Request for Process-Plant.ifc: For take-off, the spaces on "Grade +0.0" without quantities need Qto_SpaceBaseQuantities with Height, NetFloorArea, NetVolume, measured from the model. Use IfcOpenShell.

First a look at what the model holds.

```python
import ifcopenshell
import ifcopenshell.util.element
import ifcopenshell.util.unit

model = ifcopenshell.open("Process-Plant.ifc")
print(model.schema)
for unit_type in ("LENGTHUNIT", "AREAUNIT", "VOLUMEUNIT"):
    print(unit_type, ifcopenshell.util.unit.calculate_unit_scale(model, unit_type))
storey = next(s for s in model.by_type("IfcBuildingStorey") if s.Name == "Grade +0.0")
spaces = [e for e in ifcopenshell.util.element.get_decomposition(storey) if e.is_a("IfcSpace")]
for e in sorted(spaces, key=lambda e: e.id()):
    print(e.id(), e.is_a(), e.Name, list(ifcopenshell.util.element.get_psets(e, qtos_only=True)), sep=" | ")
```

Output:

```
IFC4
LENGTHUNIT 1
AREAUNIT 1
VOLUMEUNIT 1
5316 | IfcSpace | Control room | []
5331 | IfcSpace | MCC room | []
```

```python
import ifcopenshell
import ifcopenshell.api.pset
import ifcopenshell.geom
import ifcopenshell.util.element
import ifcopenshell.util.shape
import ifcopenshell.util.unit

model = ifcopenshell.open("Process-Plant.ifc")
unit_scale = ifcopenshell.util.unit.calculate_unit_scale(model)
area_scale = ifcopenshell.util.unit.calculate_unit_scale(model, "AREAUNIT")
volume_scale = ifcopenshell.util.unit.calculate_unit_scale(model, "VOLUMEUNIT")
settings = ifcopenshell.geom.settings()

storey = next(s for s in model.by_type("IfcBuildingStorey") if s.Name == "Grade +0.0")
spaces = [e for e in ifcopenshell.util.element.get_decomposition(storey) if e.is_a("IfcSpace")]

for e in sorted(spaces, key=lambda e: e.id()):
    if ifcopenshell.util.element.get_psets(e, qtos_only=True, should_inherit=False):
        continue
    # Geometry comes back in metres, in the element's own axes.
    shape = ifcopenshell.geom.create_shape(settings, e)
    values = {
        "Height": ifcopenshell.util.shape.get_z(shape.geometry) / unit_scale,
        "NetFloorArea": ifcopenshell.util.shape.get_footprint_area(shape.geometry) / area_scale,
        "NetVolume": ifcopenshell.util.shape.get_volume(shape.geometry) / volume_scale,
    }
    qto = ifcopenshell.api.pset.add_qto(model, product=e, name="Qto_SpaceBaseQuantities")
    ifcopenshell.api.pset.edit_qto(model, qto=qto, properties=values)
    print(e.id(), {k: round(v, 3) for k, v in values.items()})

model.write("Process-Plant_rev.ifc")
```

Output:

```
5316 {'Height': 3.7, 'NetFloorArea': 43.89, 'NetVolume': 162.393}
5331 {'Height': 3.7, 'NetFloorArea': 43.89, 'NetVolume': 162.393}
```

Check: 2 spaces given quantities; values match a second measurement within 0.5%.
